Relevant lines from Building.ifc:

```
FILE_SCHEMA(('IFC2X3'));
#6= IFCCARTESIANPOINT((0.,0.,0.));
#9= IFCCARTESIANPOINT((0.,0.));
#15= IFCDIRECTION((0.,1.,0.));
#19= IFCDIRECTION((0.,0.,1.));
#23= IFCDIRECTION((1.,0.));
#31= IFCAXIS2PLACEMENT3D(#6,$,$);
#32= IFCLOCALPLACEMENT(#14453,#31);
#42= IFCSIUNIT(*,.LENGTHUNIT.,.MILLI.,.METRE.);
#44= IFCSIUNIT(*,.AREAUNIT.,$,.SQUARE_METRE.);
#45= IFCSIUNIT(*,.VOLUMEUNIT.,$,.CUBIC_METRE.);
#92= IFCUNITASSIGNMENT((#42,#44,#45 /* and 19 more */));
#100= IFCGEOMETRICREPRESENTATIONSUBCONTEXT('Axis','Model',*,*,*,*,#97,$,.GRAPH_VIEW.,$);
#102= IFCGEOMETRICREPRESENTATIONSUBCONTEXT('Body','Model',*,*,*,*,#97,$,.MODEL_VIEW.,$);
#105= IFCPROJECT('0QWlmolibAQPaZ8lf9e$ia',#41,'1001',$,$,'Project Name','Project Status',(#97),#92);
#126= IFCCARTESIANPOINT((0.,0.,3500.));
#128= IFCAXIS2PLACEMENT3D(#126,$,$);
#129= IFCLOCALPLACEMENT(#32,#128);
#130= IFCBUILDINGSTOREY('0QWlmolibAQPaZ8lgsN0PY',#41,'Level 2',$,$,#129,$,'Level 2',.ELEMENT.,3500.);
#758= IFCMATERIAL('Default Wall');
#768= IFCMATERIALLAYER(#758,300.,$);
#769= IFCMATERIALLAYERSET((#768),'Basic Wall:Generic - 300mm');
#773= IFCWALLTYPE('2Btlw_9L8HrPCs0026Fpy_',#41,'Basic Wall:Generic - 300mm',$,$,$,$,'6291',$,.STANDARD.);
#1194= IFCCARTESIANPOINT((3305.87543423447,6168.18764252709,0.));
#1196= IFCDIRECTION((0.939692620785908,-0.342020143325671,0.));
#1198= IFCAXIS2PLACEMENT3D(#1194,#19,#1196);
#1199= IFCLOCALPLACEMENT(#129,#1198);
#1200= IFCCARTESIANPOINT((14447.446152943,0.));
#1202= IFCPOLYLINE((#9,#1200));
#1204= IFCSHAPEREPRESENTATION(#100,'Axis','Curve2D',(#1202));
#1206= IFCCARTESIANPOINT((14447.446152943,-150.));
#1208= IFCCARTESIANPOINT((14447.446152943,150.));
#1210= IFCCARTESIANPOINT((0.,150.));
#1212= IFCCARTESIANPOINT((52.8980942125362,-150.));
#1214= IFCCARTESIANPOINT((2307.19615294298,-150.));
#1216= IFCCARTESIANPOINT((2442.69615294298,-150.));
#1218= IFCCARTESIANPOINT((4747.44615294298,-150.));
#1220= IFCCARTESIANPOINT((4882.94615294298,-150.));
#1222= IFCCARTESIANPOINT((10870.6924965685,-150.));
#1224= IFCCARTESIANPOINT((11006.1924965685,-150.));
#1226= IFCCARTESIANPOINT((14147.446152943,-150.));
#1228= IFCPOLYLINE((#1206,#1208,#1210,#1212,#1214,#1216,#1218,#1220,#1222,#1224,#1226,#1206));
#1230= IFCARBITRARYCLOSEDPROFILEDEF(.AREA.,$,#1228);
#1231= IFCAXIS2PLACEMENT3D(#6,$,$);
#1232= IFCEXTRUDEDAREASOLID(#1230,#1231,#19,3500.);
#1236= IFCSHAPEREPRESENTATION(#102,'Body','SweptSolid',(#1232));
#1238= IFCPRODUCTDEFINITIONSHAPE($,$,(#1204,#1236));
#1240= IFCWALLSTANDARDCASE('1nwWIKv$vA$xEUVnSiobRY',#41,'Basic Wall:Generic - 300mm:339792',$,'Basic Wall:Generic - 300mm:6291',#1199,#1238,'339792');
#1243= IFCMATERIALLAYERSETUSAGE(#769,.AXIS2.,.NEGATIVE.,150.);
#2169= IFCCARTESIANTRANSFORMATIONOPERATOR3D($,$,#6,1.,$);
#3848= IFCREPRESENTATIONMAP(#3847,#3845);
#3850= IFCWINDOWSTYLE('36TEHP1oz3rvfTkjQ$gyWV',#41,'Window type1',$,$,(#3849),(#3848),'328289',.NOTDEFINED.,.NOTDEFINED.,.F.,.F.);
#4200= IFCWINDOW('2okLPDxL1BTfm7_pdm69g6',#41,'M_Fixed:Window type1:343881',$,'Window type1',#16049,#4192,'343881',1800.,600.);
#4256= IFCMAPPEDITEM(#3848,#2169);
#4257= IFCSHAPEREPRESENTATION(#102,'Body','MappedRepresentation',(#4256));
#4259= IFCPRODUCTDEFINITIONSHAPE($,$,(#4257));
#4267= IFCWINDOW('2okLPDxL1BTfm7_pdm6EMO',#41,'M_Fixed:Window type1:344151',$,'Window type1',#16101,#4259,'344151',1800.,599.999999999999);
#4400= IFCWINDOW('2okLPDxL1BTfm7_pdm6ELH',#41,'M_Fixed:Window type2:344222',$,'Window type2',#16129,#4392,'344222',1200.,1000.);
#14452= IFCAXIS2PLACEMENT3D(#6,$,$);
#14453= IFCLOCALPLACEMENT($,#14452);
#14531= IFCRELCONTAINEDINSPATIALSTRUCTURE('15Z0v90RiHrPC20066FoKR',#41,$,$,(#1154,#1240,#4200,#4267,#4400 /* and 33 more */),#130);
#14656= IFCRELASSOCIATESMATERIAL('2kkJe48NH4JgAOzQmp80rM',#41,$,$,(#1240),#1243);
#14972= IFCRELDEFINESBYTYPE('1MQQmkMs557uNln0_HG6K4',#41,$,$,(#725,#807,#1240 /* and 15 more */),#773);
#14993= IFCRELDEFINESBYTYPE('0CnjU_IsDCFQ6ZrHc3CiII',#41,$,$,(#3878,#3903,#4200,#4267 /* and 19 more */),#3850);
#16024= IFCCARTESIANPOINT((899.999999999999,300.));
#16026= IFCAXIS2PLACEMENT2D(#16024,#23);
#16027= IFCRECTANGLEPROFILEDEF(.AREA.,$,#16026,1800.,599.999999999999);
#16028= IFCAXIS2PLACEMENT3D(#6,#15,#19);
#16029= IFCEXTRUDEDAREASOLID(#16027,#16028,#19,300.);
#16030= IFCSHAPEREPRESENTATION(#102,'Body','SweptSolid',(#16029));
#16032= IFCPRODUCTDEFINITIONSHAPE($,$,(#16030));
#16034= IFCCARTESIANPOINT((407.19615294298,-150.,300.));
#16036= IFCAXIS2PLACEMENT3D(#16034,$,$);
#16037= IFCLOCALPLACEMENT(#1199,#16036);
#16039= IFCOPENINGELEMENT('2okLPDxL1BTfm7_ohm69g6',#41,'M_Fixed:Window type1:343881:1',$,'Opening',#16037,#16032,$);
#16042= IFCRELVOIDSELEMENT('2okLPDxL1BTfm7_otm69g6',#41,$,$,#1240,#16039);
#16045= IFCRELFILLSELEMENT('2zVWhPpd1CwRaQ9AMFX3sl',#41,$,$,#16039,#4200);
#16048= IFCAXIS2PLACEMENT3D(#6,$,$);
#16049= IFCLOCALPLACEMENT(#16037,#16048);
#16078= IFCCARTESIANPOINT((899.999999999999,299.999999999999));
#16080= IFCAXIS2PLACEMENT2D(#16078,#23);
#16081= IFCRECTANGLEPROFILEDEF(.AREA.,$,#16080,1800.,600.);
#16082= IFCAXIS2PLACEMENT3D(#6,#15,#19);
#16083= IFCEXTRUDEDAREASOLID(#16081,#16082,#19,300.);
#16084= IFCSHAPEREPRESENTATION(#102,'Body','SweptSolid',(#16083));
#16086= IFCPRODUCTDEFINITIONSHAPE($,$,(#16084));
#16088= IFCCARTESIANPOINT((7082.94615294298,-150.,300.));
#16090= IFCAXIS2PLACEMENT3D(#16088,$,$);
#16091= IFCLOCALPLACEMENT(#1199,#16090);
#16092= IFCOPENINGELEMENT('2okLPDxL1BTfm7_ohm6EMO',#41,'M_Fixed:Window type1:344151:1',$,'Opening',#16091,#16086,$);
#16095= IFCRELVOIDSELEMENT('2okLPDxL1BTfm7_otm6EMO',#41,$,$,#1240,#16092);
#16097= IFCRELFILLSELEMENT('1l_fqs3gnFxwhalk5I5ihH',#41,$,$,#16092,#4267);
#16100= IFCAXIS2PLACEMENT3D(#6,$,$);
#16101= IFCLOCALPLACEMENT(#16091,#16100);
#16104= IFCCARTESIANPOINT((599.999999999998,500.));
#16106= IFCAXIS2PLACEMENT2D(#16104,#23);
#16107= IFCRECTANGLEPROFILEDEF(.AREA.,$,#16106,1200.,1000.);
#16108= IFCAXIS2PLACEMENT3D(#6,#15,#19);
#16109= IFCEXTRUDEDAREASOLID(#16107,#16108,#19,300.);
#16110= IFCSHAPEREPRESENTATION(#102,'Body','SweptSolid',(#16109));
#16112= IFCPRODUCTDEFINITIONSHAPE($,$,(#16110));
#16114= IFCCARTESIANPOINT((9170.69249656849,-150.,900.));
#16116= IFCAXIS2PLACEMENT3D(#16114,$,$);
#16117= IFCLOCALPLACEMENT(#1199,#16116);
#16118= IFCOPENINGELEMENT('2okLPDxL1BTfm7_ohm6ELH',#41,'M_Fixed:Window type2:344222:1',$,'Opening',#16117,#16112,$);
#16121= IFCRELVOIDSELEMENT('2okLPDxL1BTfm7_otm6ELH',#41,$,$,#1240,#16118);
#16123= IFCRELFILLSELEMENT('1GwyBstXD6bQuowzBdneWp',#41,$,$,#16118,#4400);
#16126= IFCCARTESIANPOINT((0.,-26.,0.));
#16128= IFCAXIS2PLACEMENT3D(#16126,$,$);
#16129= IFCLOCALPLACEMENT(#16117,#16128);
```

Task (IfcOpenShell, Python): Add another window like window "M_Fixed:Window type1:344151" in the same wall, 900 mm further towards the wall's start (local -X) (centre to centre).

```python
import ifcopenshell
import ifcopenshell.api.feature
import ifcopenshell.api.geometry
import ifcopenshell.api.root
import ifcopenshell.geom
import ifcopenshell.util.element
import ifcopenshell.util.placement
import ifcopenshell.util.shape
import ifcopenshell.util.unit

model = ifcopenshell.open("Building.ifc")
unit_scale = ifcopenshell.util.unit.calculate_unit_scale(model)
settings = ifcopenshell.geom.settings()


def volume(element):
    """Net volume in cubic metres, openings subtracted."""
    shape = ifcopenshell.geom.create_shape(settings, element)
    return ifcopenshell.util.shape.get_volume(shape.geometry)


def reuse_history(source, copy):
    """copy_class also copies each property set's owner history, people and application; keep the originals."""
    for rel in copy.IsDefinedBy:
        if rel.is_a("IfcRelDefinesByProperties") and (history := rel.RelatingPropertyDefinition.OwnerHistory):
            rel.RelatingPropertyDefinition.OwnerHistory = source.OwnerHistory
            ifcopenshell.util.element.remove_deep2(model, history)


window = model.by_id(4267)
opening = window.FillsVoids[0].RelatingOpeningElement
wall = opening.VoidsElements[0].RelatingBuildingElement
before = volume(wall)
shift = ifcopenshell.util.placement.get_local_placement(wall.ObjectPlacement)[:3, 0] * -0.9 / unit_scale

# copy_class copies the void relationship, type, container and properties, but no geometry.
new_opening = ifcopenshell.api.root.copy_class(model, product=opening)
new_opening.Representation = ifcopenshell.util.element.copy_deep(
    model, opening.Representation, exclude=["IfcGeometricRepresentationContext", "IfcRepresentationMap"]
)
new_opening.Name = "M_Fixed:Window type1"
new_window = ifcopenshell.api.root.copy_class(model, product=window)
new_window.Representation = ifcopenshell.util.element.copy_deep(
    model, window.Representation, exclude=["IfcGeometricRepresentationContext", "IfcRepresentationMap"]
)
new_window.Name = "M_Fixed:Window type1"
new_window.Tag = None
reuse_history(window, new_window)
fills = ifcopenshell.api.feature.add_filling(model, opening=new_opening, element=new_window)
fills.OwnerHistory = new_window.OwnerHistory  # required in IFC2X3

for old, new in ((opening, new_opening), (window, new_window)):
    matrix = ifcopenshell.util.placement.get_local_placement(old.ObjectPlacement)
    matrix[:3, 3] += shift
    ifcopenshell.api.geometry.edit_object_placement(model, product=new, matrix=matrix, is_si=False)

after = volume(wall)

print(f"wall volume {before:.3f} -> {after:.3f} m3")

model.write("Building_rev.ifc")
```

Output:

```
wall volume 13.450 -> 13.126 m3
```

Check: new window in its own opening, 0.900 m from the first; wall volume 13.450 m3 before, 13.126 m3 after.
